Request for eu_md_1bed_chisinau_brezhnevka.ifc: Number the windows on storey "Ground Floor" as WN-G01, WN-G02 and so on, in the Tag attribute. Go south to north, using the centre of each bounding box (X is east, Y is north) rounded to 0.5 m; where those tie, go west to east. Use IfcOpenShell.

First a look at what the model holds.

```python
import ifcopenshell
import ifcopenshell.util.element
import ifcopenshell.util.placement

model = ifcopenshell.open("eu_md_1bed_chisinau_brezhnevka.ifc")
print(model.schema)
storey = next(s for s in model.by_type("IfcBuildingStorey") if s.Name == "Ground Floor")
windows = [e for e in ifcopenshell.util.element.get_decomposition(storey) if e.is_a("IfcWindow")]
for e in sorted(windows, key=lambda e: e.id()):
    origin = ifcopenshell.util.placement.get_local_placement(e.ObjectPlacement)[:3, 3]
    print(e.id(), e.Tag, e.Name, origin.round(2) + 0.0, sep=" | ")
```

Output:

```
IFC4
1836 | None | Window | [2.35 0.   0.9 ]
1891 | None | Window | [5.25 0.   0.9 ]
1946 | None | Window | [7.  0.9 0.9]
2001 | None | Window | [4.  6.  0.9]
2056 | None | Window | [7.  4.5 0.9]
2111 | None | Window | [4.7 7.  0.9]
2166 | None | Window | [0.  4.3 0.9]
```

```python
import ifcopenshell
import ifcopenshell.geom
import ifcopenshell.util.element
import ifcopenshell.util.shape

model = ifcopenshell.open("eu_md_1bed_chisinau_brezhnevka.ifc")
settings = ifcopenshell.geom.settings()
settings.set("use-world-coords", True)


def centre(element):
    shape = ifcopenshell.geom.create_shape(settings, element)
    return ifcopenshell.util.shape.get_bbox_centroid(shape.geometry)


storey = next(s for s in model.by_type("IfcBuildingStorey") if s.Name == "Ground Floor")
windows = [e for e in ifcopenshell.util.element.get_decomposition(storey) if e.is_a("IfcWindow")]

# Insertion points can sit at a corner or the storey origin, so sort by the geometry (in metres).
centres = {e: centre(e) for e in windows}
windows.sort(key=lambda e: (round(centres[e][1] / 0.5), centres[e][0]))

for i, e in enumerate(windows, start=1):
    number = f"WN-G{i:02d}"
    e.Tag = number
    print(e.id(), number)

model.write("eu_md_1bed_chisinau_brezhnevka_edited.ifc")
```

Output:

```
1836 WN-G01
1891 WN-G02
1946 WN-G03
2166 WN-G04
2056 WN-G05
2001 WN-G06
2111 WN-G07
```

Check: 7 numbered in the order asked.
